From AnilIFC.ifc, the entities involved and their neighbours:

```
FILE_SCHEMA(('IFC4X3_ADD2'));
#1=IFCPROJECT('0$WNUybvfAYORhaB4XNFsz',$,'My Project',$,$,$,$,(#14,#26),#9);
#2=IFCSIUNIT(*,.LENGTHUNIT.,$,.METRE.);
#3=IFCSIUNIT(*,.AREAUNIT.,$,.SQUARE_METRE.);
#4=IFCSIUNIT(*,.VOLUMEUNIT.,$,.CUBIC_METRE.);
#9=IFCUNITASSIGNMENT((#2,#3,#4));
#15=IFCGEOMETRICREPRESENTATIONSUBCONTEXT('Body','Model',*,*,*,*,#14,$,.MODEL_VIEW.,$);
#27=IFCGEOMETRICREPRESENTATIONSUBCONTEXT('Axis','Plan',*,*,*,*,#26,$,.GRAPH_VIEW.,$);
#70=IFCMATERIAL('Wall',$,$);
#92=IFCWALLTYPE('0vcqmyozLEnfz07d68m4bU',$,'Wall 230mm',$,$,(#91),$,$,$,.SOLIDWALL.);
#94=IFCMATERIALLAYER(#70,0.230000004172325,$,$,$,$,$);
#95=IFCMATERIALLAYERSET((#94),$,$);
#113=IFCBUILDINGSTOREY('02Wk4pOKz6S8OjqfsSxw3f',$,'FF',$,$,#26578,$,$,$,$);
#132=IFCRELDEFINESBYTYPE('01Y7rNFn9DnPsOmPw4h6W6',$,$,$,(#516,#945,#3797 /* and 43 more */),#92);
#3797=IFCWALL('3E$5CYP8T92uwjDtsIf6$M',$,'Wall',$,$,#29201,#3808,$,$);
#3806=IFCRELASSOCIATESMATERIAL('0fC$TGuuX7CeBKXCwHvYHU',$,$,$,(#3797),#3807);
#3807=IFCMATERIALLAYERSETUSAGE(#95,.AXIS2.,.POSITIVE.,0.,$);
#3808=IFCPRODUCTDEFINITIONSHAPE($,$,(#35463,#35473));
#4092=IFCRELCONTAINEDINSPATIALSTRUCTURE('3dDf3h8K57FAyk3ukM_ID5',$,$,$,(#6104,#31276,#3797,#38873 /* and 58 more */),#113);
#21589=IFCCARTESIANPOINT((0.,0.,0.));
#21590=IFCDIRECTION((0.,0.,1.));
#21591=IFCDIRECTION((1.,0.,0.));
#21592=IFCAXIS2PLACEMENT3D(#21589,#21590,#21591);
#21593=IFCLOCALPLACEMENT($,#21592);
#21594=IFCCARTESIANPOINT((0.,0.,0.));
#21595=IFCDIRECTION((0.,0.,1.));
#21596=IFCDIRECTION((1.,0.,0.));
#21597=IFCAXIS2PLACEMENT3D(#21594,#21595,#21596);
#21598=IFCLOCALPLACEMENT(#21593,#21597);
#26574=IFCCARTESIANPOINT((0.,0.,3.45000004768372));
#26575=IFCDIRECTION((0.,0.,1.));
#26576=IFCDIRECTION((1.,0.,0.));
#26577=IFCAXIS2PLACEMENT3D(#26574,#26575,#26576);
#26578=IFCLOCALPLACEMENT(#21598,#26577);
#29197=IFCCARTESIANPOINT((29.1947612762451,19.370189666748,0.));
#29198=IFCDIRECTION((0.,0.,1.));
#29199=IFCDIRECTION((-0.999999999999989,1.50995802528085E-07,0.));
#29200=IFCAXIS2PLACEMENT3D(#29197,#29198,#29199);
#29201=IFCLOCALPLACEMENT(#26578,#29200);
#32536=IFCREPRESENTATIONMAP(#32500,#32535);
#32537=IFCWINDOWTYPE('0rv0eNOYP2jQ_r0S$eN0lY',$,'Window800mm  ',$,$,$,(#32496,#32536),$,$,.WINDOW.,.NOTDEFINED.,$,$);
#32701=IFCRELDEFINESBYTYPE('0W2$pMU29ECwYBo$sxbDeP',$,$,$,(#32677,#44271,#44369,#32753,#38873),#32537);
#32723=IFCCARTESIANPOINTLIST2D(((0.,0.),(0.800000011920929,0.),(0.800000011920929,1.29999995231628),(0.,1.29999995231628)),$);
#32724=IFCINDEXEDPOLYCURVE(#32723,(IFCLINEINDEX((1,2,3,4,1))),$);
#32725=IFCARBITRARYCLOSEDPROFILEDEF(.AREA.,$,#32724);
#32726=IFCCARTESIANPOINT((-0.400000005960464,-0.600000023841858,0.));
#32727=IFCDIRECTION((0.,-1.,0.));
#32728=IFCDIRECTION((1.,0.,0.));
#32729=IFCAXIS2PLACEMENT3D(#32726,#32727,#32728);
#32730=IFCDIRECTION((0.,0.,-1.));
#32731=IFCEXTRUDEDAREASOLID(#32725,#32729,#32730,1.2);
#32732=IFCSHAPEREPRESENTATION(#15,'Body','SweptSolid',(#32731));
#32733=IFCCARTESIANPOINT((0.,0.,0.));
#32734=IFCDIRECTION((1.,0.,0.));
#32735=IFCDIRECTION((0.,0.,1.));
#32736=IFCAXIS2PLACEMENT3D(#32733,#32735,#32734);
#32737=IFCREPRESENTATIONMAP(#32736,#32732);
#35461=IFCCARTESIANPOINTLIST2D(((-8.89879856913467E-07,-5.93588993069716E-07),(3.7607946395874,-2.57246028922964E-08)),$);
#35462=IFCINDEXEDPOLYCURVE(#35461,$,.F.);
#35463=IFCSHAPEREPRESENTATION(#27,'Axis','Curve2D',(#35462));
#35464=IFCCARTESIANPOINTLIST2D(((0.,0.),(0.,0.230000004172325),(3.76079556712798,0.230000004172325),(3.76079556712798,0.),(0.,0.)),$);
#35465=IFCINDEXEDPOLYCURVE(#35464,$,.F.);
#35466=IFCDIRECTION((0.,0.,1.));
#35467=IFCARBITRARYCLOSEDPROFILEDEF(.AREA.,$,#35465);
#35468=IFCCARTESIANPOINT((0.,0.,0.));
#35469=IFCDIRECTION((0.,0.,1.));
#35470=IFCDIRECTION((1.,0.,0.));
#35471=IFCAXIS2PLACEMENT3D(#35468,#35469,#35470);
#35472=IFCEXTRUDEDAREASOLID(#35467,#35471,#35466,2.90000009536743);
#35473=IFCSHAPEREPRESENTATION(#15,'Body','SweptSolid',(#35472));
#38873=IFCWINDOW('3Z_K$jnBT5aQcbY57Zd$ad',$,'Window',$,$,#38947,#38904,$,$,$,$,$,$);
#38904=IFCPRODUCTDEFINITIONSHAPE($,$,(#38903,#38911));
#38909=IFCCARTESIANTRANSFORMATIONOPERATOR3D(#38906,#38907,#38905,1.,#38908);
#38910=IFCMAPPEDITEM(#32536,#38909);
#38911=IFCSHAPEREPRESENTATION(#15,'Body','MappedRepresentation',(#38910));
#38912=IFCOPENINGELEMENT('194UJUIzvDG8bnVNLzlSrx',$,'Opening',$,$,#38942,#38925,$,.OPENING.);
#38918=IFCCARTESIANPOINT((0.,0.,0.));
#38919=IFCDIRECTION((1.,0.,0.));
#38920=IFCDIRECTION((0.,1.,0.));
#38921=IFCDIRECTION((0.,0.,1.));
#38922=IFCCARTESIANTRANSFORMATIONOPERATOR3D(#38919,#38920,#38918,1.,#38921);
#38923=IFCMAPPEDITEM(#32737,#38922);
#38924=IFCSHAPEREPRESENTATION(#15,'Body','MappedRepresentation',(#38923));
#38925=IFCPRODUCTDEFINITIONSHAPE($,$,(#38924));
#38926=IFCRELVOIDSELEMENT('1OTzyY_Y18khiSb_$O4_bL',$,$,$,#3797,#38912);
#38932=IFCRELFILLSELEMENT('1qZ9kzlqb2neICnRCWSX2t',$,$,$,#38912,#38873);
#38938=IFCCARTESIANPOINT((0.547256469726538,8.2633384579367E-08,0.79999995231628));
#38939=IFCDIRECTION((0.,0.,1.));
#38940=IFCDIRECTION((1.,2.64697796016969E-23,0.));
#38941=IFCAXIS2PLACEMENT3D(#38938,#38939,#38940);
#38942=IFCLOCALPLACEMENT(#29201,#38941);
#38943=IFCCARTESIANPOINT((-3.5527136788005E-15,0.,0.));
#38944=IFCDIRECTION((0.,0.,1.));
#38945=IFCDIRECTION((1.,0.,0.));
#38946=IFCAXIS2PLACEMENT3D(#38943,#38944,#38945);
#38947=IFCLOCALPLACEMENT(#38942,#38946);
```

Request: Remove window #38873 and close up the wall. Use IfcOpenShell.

```python
import ifcopenshell
import ifcopenshell.api.feature
import ifcopenshell.api.root
import ifcopenshell.geom
import ifcopenshell.util.shape

model = ifcopenshell.open("AnilIFC.ifc")
settings = ifcopenshell.geom.settings()


def volume(element):
    """Net volume in cubic metres, openings subtracted."""
    shape = ifcopenshell.geom.create_shape(settings, element)
    return ifcopenshell.util.shape.get_volume(shape.geometry)


window = model.by_id(38873)
opening = window.FillsVoids[0].RelatingOpeningElement
wall = opening.VoidsElements[0].RelatingBuildingElement
before = volume(wall)

ifcopenshell.api.root.remove_product(model, product=window)
ifcopenshell.api.feature.remove_feature(model, feature=opening)

after = volume(wall)

print(f"wall volume {before:.3f} -> {after:.3f} m3")

model.write("AnilIFC_edited.ifc")
```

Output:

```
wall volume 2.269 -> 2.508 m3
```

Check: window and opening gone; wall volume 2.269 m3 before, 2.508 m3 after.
